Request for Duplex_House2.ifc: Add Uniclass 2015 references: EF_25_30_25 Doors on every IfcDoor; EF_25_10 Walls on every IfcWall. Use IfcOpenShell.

First a look at what the model holds.

```python
import ifcopenshell

model = ifcopenshell.open("Duplex_House2.ifc")
print(model.schema)
print("classifications:", [c.Name for c in model.by_type("IfcClassification")])
for ifc_class in ("IfcDoor", "IfcRoof", "IfcStair", "IfcWall", "IfcWindow"):
    print(ifc_class, len(model.by_type(ifc_class)))
```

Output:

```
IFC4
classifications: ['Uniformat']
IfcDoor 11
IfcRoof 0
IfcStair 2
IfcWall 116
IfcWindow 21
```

```python
import ifcopenshell
import ifcopenshell.api.classification

model = ifcopenshell.open("Duplex_House2.ifc")

system = ifcopenshell.api.classification.add_classification(model, classification="Uniclass 2015")

codes = {
    "IfcDoor": ("EF_25_30_25", "Doors"),
    "IfcWall": ("EF_25_10", "Walls"),
}
for ifc_class, (code, name) in codes.items():
    products = model.by_type(ifc_class)
    ifcopenshell.api.classification.add_reference(
        model, products=products, classification=system, identification=code, name=name
    )
    print(code, len(products))

model.write("Duplex_House2-out.ifc")
```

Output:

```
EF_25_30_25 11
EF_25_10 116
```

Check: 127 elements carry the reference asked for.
